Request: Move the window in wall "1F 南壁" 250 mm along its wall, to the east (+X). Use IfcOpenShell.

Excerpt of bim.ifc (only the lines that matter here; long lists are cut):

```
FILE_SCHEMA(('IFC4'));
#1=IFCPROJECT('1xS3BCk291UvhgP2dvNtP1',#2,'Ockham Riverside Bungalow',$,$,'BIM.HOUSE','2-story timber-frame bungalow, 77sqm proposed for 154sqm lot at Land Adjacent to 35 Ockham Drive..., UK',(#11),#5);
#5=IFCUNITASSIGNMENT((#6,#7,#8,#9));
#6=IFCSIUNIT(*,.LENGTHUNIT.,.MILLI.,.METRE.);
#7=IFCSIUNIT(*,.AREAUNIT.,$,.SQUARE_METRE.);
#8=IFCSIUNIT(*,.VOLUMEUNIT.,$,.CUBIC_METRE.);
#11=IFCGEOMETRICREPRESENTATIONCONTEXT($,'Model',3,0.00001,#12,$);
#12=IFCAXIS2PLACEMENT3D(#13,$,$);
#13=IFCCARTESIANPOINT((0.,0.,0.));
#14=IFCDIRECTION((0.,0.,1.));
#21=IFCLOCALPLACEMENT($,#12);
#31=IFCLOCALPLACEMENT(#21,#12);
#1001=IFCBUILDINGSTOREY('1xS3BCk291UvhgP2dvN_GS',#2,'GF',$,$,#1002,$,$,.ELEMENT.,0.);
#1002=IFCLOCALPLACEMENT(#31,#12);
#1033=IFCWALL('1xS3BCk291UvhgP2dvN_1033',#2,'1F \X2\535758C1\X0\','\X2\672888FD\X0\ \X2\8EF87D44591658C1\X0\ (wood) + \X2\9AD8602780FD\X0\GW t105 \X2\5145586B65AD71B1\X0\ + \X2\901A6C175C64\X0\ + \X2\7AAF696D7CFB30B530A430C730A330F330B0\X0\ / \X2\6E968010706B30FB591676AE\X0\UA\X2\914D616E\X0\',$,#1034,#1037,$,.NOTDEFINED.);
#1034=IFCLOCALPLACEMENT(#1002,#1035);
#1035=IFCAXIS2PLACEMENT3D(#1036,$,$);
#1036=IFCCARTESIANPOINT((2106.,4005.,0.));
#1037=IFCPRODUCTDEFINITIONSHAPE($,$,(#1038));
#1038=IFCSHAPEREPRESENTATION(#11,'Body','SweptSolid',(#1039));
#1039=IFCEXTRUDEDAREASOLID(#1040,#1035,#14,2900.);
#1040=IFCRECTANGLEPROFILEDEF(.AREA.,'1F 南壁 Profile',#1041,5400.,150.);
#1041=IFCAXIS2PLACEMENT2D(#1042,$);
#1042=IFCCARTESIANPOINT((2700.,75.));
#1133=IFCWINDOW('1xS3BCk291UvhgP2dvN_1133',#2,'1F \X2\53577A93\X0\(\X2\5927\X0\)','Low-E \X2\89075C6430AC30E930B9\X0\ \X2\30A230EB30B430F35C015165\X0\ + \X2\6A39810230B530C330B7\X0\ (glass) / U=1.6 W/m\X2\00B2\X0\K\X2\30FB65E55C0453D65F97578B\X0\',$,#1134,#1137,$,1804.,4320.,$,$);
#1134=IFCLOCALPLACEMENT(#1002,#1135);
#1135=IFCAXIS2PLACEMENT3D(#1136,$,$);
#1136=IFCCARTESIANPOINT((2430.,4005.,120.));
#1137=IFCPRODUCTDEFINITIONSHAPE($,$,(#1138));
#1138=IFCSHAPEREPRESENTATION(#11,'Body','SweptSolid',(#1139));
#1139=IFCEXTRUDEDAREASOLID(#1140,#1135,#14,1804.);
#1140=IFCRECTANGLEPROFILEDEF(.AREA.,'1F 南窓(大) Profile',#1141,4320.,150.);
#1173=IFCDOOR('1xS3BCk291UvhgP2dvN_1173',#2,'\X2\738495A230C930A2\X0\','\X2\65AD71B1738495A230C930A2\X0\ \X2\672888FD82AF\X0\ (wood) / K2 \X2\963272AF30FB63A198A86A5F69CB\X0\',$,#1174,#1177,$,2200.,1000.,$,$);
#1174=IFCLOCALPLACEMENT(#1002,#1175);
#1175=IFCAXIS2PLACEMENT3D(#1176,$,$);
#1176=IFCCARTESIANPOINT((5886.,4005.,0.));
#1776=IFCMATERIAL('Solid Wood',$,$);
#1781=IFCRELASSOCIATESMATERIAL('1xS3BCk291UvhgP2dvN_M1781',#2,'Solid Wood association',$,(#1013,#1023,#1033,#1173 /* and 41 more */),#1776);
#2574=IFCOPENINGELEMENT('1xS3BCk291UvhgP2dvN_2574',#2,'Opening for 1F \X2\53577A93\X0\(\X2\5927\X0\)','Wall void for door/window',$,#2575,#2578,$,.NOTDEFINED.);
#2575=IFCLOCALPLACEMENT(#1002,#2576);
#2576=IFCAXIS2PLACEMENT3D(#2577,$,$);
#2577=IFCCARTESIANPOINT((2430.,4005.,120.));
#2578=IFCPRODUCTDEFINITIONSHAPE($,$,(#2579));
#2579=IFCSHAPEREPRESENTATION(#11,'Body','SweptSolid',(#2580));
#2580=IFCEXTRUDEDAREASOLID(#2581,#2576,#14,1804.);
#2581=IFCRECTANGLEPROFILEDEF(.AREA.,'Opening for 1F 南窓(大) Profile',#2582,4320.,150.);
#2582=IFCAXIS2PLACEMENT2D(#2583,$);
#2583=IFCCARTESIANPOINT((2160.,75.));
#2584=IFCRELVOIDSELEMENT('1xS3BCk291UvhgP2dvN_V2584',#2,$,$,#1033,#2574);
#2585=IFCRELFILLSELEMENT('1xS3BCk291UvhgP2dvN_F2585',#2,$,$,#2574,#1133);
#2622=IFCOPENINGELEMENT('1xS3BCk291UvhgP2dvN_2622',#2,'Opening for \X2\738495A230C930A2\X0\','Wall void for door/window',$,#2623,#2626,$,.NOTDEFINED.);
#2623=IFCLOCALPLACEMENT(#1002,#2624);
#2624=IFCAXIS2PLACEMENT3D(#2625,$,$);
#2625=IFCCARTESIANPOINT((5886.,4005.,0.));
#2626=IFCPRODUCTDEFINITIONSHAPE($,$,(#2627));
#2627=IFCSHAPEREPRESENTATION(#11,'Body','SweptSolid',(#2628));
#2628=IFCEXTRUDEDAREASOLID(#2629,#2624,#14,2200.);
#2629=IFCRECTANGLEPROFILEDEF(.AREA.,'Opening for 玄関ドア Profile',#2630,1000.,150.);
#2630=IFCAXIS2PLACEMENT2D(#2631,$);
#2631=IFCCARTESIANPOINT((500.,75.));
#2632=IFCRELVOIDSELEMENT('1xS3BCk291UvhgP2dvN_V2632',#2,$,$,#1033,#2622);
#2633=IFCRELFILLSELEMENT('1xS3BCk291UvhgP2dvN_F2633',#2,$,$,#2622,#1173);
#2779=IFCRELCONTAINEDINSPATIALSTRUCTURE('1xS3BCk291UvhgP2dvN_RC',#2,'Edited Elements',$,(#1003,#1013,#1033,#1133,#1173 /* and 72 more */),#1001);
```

```python
import ifcopenshell
import ifcopenshell.api.geometry
import ifcopenshell.util.placement

model = ifcopenshell.open("bim.ifc")

window = model.by_id(1133)
opening = window.FillsVoids[0].RelatingOpeningElement
wall = opening.VoidsElements[0].RelatingBuildingElement

wall_matrix = ifcopenshell.util.placement.get_local_placement(wall.ObjectPlacement)
shift = wall_matrix[:3, 0] * 250.0
before = ifcopenshell.util.placement.get_local_placement(window.ObjectPlacement)[:3, 3].copy()

# The window is not placed relative to its opening, so move both.
for product in (opening, window):
    matrix = ifcopenshell.util.placement.get_local_placement(product.ObjectPlacement)
    matrix[:3, 3] += shift
    ifcopenshell.api.geometry.edit_object_placement(model, product=product, matrix=matrix, is_si=False)

after = ifcopenshell.util.placement.get_local_placement(window.ObjectPlacement)[:3, 3]
print("window moved by", (after - before).round(3) + 0.0)

model.write("bim_rev.ifc")
```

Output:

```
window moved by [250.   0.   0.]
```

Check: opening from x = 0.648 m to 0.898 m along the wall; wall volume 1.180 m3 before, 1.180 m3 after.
